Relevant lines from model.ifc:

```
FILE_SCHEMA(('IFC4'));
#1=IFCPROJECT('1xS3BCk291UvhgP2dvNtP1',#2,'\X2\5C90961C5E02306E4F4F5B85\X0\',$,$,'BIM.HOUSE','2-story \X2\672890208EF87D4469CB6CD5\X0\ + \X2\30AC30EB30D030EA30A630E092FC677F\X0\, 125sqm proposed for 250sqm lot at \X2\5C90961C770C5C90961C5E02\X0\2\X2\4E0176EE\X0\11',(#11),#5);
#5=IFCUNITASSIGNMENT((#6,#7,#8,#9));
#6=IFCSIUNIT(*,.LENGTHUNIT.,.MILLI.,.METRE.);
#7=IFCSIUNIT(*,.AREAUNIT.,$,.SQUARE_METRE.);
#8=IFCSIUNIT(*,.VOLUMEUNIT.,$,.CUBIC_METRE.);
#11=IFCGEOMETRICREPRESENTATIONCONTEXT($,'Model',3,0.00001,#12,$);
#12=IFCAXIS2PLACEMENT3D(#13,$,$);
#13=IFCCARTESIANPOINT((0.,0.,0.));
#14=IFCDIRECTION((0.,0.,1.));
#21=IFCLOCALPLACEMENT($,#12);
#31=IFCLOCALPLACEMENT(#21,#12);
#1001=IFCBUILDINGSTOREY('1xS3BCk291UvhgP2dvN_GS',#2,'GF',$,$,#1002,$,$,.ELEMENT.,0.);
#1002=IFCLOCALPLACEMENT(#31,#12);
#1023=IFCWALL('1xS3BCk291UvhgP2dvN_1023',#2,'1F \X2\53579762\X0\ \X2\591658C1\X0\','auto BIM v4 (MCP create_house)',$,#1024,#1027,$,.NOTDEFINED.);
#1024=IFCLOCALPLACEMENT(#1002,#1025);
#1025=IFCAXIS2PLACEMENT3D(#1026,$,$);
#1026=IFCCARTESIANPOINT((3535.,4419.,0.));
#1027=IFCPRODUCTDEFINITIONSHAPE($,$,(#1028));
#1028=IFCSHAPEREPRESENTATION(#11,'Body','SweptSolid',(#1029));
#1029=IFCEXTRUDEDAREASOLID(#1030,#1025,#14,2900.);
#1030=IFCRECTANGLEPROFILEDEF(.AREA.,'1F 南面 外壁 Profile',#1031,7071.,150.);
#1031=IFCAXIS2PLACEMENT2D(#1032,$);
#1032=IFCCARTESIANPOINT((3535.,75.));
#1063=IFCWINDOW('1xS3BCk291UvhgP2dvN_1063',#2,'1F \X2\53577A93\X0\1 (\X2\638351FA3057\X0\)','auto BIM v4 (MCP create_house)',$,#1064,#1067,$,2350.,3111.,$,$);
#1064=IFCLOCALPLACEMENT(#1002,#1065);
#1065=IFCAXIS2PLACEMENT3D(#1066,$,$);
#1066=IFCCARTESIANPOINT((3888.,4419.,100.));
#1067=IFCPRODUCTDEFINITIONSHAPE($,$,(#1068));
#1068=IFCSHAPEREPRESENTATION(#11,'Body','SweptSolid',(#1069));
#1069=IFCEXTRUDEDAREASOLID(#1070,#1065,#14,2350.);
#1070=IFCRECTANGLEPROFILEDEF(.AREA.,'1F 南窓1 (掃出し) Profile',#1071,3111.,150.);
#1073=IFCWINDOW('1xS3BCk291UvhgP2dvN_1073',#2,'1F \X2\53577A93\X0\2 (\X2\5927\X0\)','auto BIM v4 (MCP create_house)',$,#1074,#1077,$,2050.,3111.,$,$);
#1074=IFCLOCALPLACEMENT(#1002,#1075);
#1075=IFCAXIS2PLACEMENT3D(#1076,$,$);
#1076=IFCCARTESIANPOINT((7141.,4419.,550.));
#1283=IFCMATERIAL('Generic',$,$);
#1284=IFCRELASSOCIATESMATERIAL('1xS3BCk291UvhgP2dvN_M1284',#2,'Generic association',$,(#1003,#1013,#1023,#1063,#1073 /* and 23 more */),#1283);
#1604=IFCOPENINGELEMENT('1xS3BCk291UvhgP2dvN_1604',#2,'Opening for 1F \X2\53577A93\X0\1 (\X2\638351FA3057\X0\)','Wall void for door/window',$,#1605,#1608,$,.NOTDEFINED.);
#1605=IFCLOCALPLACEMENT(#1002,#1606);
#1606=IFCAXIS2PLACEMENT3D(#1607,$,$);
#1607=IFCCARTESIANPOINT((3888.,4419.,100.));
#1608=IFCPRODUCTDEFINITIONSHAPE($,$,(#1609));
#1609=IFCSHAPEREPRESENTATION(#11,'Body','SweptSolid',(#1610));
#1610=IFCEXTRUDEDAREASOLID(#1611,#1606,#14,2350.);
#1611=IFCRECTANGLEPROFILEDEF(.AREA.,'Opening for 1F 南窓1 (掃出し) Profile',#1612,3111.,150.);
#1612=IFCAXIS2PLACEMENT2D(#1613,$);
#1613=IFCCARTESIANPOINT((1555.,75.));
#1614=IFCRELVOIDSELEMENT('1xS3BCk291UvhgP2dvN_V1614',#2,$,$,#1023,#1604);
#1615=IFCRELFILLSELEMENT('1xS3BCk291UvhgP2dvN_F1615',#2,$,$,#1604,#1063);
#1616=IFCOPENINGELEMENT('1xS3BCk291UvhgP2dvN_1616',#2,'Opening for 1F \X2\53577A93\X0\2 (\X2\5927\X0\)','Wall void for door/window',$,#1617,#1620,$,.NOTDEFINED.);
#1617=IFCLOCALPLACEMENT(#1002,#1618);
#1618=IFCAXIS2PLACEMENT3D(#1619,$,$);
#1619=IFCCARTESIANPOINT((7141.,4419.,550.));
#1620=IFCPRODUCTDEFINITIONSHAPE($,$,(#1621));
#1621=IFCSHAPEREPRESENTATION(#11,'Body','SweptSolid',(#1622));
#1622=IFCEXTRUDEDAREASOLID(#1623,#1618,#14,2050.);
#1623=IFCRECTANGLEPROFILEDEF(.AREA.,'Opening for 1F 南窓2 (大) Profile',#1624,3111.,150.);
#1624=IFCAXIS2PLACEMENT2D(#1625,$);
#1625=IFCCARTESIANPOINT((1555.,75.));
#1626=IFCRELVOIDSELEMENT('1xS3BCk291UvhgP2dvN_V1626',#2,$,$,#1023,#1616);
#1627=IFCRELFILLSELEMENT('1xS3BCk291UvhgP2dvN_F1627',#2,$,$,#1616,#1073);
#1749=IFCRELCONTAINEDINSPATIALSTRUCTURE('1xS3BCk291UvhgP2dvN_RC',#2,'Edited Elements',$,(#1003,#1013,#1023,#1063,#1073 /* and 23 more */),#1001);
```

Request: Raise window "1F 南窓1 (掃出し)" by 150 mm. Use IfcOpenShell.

```python
import numpy as np
import ifcopenshell
import ifcopenshell.api.geometry
import ifcopenshell.util.placement
import ifcopenshell.util.unit

model = ifcopenshell.open("model.ifc")
unit_scale = ifcopenshell.util.unit.calculate_unit_scale(model)

window = model.by_guid("1xS3BCk291UvhgP2dvN_1063")
opening = window.FillsVoids[0].RelatingOpeningElement
dz = 150.0

shift = np.array([0.0, 0.0, dz])
# The window is not placed relative to its opening, so move both.
for product in (opening, window):
    matrix = ifcopenshell.util.placement.get_local_placement(product.ObjectPlacement)
    matrix[:3, 3] += shift
    ifcopenshell.api.geometry.edit_object_placement(model, product=product, matrix=matrix, is_si=False)

print(f"moved by {dz * unit_scale:+.3f} m")

model.write("model_updated.ifc")
```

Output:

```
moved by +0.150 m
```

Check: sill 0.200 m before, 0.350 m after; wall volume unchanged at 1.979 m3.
